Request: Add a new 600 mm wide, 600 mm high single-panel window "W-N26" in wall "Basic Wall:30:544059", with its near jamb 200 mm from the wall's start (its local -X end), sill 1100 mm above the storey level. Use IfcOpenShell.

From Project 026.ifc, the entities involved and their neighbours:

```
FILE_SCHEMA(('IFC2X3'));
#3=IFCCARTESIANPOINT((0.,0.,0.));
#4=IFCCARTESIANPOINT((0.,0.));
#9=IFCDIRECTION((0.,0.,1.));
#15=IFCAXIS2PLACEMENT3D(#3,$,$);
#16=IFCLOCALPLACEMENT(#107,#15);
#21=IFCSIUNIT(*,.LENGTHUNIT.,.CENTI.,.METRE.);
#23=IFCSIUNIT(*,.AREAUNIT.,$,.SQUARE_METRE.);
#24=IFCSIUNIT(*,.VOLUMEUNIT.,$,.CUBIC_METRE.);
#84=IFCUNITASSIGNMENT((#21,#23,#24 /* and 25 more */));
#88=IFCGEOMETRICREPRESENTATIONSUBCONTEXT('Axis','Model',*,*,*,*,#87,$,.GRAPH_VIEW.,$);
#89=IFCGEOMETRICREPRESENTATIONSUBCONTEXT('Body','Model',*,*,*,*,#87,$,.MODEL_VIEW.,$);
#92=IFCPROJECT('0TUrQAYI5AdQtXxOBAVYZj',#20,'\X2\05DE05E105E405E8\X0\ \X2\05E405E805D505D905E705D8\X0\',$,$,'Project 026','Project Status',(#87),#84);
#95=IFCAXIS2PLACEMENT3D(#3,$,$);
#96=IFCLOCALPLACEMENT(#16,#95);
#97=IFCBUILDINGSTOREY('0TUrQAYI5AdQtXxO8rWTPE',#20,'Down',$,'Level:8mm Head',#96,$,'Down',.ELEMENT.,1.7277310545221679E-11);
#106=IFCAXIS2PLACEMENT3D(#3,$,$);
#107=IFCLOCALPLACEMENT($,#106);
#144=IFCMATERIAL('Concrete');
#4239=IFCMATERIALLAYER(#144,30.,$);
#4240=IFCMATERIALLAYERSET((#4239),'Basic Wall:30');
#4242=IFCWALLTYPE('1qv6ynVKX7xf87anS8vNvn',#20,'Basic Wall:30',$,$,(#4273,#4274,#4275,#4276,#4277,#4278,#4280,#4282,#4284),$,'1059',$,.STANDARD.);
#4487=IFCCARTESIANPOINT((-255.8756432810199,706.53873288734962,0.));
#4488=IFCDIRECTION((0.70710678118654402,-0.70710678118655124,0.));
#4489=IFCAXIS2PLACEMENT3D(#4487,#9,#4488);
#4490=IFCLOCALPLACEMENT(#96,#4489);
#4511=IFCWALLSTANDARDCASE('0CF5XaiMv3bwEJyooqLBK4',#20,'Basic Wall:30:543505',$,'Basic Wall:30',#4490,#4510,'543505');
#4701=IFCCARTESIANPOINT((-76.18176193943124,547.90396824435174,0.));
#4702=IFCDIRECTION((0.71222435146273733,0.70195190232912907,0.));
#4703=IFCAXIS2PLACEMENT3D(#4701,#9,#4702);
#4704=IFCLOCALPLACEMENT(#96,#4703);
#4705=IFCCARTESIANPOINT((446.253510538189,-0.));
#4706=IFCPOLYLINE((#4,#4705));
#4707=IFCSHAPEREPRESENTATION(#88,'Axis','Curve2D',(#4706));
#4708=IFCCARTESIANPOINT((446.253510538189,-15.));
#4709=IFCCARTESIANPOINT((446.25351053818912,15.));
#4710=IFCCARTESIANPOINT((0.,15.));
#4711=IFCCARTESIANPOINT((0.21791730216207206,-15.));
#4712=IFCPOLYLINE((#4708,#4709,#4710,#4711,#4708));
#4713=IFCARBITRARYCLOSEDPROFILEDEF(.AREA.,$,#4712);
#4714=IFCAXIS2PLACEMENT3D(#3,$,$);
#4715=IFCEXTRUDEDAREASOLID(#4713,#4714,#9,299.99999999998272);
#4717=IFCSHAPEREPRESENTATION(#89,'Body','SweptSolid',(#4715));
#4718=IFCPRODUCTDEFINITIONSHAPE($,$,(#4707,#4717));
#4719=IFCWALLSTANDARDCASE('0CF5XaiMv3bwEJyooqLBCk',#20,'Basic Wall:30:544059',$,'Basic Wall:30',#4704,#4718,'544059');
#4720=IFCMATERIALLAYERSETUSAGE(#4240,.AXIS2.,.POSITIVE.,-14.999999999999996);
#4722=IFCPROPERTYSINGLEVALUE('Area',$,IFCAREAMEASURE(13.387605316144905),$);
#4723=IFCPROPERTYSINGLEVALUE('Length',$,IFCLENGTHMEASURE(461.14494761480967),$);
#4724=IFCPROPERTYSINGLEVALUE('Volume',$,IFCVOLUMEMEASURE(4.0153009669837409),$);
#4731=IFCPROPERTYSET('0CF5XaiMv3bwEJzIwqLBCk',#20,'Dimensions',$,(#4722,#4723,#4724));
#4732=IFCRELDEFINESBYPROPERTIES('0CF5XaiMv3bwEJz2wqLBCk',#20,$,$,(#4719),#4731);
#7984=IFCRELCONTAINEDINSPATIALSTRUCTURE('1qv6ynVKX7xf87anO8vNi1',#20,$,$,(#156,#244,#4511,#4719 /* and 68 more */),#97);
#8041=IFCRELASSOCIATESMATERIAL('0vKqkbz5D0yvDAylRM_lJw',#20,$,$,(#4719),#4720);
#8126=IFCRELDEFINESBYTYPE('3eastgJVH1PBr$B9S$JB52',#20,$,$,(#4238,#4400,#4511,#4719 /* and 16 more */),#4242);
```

```python
import numpy as np
import ifcopenshell
import ifcopenshell.api.feature
import ifcopenshell.api.geometry
import ifcopenshell.api.pset
import ifcopenshell.api.root
import ifcopenshell.api.spatial
import ifcopenshell.api.type
import ifcopenshell.geom
import ifcopenshell.util.element
import ifcopenshell.util.placement
import ifcopenshell.util.representation
import ifcopenshell.util.shape
import ifcopenshell.util.unit

model = ifcopenshell.open("Project 026.ifc")
unit_scale = ifcopenshell.util.unit.calculate_unit_scale(model)
area_scale = ifcopenshell.util.unit.calculate_unit_scale(model, "AREAUNIT")
volume_scale = ifcopenshell.util.unit.calculate_unit_scale(model, "VOLUMEUNIT")
settings = ifcopenshell.geom.settings()


def volume(element):
    """Net volume in cubic metres, openings subtracted."""
    shape = ifcopenshell.geom.create_shape(settings, element)
    return ifcopenshell.util.shape.get_volume(shape.geometry)


wall = model.by_id(4719)
storey = ifcopenshell.util.element.get_container(wall, ifc_class="IfcBuildingStorey")
context = ifcopenshell.util.representation.get_context(model, "Model", "Body", "MODEL_VIEW")
before = volume(wall)

width, height, from_end, sill = 0.6, 0.6, 0.2, 1.1  # metres

# The wall runs along its own X axis, and the end named is its -X end.
wall_shape = ifcopenshell.geom.create_shape(settings, wall)
x, y, z = ifcopenshell.util.shape.get_vertices(wall_shape.geometry).T
start = x.min() + from_end
face, thickness = float(y.min()), float(y.max() - y.min())
wall_matrix = ifcopenshell.util.placement.get_local_placement(wall.ObjectPlacement)
level = ifcopenshell.util.placement.get_local_placement(storey.ObjectPlacement)[2, 3]


def in_wall(x, y):
    """Placement at x, y metres in the wall's axes, at sill height."""
    matrix = wall_matrix.copy()
    matrix[:, 3] = wall_matrix @ np.array([x / unit_scale, y / unit_scale, 0.0, 1.0])
    matrix[2, 3] = level + sill / unit_scale
    return matrix


# Opening: a box that overshoots both wall faces by 50 mm.
opening = ifcopenshell.api.root.create_entity(model, ifc_class="IfcOpeningElement")
box = ifcopenshell.api.geometry.add_wall_representation(
    model, context=context, length=width, height=height, thickness=thickness + 0.1
)
ifcopenshell.api.geometry.assign_representation(model, product=opening, representation=box)
ifcopenshell.api.geometry.edit_object_placement(model, product=opening, matrix=in_wall(start, face - 0.05), is_si=False)
ifcopenshell.api.feature.add_feature(model, feature=opening, element=wall)

window = ifcopenshell.api.root.create_entity(model, ifc_class="IfcWindow", name="W-N26")
window.OverallWidth, window.OverallHeight = width / unit_scale, height / unit_scale
body = ifcopenshell.api.geometry.add_window_representation(
    model,
    context=context,
    overall_width=window.OverallWidth,
    overall_height=window.OverallHeight,
    partition_type="SINGLE_PANEL",
)
ifcopenshell.api.geometry.assign_representation(model, product=window, representation=body)
ifcopenshell.api.spatial.assign_container(model, products=[window], relating_structure=storey)
fills = ifcopenshell.api.feature.add_filling(model, opening=opening, element=window)
fills.OwnerHistory = window.OwnerHistory  # required in IFC2X3

# IFC2X3 keeps the operation on the window style.
style = ifcopenshell.api.root.create_entity(model, ifc_class="IfcWindowStyle", name="W-N26")
style.OperationType, style.ConstructionType = "SINGLE_PANEL", "NOTDEFINED"
style.ParameterTakesPrecedence = style.Sizeable = False
ifcopenshell.api.type.assign_type(model, related_objects=[window], relating_type=style)

# Centre the window in the wall's thickness.
ifcopenshell.api.geometry.edit_object_placement(model, product=window, matrix=in_wall(start, face), is_si=False)
window_shape = ifcopenshell.geom.create_shape(settings, window)
depth = ifcopenshell.util.shape.get_vertices(window_shape.geometry)[:, 1]
offset = face + thickness / 2 - (depth.min() + depth.max()) / 2
ifcopenshell.api.geometry.edit_object_placement(model, product=window, matrix=in_wall(start, offset), is_si=False)

after = volume(wall)

# Update the wall's stored quantities.
pset = model.by_id(ifcopenshell.util.element.get_pset(wall, "Dimensions", should_inherit=False)["id"])
ifcopenshell.api.pset.edit_pset(model, pset=pset, properties={
    "Area": model.create_entity("IfcAreaMeasure", after / thickness / area_scale),
    "Volume": model.create_entity("IfcVolumeMeasure", after / volume_scale),
})

print(f"wall volume {before:.3f} -> {after:.3f} m3")

model.write("Project 026_edited.ifc")
```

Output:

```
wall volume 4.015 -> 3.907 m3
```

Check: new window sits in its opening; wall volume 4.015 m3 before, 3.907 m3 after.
